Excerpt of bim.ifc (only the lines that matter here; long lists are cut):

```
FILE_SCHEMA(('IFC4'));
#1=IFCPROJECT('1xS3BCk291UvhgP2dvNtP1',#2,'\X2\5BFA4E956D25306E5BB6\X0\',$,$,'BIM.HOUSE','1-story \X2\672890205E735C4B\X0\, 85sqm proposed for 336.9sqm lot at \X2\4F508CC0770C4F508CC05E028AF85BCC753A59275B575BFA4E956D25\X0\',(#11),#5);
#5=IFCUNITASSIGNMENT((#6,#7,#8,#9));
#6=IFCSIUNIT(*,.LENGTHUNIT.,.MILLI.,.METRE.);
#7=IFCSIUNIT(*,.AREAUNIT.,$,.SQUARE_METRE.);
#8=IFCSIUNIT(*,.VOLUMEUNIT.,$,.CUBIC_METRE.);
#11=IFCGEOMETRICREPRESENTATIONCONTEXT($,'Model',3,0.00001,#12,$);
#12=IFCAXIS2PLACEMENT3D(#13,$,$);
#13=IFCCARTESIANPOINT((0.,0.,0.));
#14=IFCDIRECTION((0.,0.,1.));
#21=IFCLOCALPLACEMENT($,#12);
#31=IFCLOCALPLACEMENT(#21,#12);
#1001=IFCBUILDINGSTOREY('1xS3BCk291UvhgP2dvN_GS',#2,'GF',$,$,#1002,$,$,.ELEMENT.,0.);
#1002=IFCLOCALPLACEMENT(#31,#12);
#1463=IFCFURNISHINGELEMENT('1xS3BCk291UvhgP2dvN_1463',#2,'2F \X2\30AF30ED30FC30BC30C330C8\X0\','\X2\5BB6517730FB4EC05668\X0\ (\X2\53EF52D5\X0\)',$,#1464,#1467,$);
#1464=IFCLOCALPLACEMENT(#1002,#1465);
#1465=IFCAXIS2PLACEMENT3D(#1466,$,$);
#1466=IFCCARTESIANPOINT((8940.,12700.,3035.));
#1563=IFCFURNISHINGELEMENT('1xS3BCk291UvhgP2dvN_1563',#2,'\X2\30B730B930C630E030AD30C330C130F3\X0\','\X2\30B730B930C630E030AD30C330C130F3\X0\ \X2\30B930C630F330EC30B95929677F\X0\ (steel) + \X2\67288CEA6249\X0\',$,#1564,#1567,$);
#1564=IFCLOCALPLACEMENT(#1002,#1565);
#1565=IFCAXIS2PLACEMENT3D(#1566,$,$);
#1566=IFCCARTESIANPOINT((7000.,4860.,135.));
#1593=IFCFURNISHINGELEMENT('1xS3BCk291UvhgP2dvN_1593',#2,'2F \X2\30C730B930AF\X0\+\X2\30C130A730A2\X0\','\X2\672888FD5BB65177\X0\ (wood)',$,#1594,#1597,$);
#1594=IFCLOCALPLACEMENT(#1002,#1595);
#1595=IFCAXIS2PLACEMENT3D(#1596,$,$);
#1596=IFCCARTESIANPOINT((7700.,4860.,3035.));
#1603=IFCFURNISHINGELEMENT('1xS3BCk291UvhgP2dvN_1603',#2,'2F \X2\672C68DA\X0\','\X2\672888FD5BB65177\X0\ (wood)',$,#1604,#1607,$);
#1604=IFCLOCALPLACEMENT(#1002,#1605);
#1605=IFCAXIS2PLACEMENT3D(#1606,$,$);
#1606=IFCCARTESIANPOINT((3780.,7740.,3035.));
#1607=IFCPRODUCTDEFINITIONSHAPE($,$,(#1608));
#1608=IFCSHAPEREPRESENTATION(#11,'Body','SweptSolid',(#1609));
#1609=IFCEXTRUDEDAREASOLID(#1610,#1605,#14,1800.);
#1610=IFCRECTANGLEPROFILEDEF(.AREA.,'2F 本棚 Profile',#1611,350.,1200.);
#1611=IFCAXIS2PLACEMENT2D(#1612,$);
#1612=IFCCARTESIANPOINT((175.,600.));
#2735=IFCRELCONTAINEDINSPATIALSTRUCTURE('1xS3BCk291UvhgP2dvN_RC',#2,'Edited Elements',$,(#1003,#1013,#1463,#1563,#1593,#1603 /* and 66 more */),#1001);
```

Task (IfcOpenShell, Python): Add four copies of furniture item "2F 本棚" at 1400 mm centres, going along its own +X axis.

```python
import ifcopenshell
import ifcopenshell.api.geometry
import ifcopenshell.api.root
import ifcopenshell.util.element
import ifcopenshell.util.placement
import ifcopenshell.util.unit

model = ifcopenshell.open("bim.ifc")
unit_scale = ifcopenshell.util.unit.calculate_unit_scale(model)


def reuse_history(source, copy):
    """copy_class also copies each property set's owner history, people and application; keep the originals."""
    for rel in copy.IsDefinedBy:
        if rel.is_a("IfcRelDefinesByProperties") and (history := rel.RelatingPropertyDefinition.OwnerHistory):
            rel.RelatingPropertyDefinition.OwnerHistory = source.OwnerHistory
            ifcopenshell.util.element.remove_deep2(model, history)


source = model.by_guid("1xS3BCk291UvhgP2dvN_1603")
base = ifcopenshell.util.placement.get_local_placement(source.ObjectPlacement)
step = base[:3, 0] * 1.4 / unit_scale

for i in range(1, 5):
    copy = ifcopenshell.api.root.copy_class(model, product=source)
    copy.Representation = ifcopenshell.util.element.copy_deep(
        model, source.Representation, exclude=["IfcGeometricRepresentationContext", "IfcRepresentationMap"]
    )
    reuse_history(source, copy)
    matrix = base.copy()
    matrix[:3, 3] += i * step
    print("added at", matrix[:3, 3].round(3) + 0.0)
    ifcopenshell.api.geometry.edit_object_placement(model, product=copy, matrix=matrix, is_si=False)

model.write("bim_rev.ifc")
```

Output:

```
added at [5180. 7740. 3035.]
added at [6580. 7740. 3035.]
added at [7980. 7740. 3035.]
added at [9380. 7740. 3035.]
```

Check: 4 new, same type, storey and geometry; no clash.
